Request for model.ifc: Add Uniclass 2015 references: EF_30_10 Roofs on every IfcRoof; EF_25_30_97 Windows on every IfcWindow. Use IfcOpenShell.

First a look at what the model holds.

```python
import ifcopenshell

model = ifcopenshell.open("model.ifc")
print(model.schema)
print("classifications:", [c.Name for c in model.by_type("IfcClassification")])
for ifc_class in ("IfcDoor", "IfcRoof", "IfcStair", "IfcWall", "IfcWindow"):
    print(ifc_class, len(model.by_type(ifc_class)))
```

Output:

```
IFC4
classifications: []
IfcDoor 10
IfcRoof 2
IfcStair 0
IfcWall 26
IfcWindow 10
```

```python
import ifcopenshell
import ifcopenshell.api.classification

model = ifcopenshell.open("model.ifc")

system = ifcopenshell.api.classification.add_classification(model, classification="Uniclass 2015")

codes = {
    "IfcRoof": ("EF_30_10", "Roofs"),
    "IfcWindow": ("EF_25_30_97", "Windows"),
}
for ifc_class, (code, name) in codes.items():
    products = model.by_type(ifc_class)
    ifcopenshell.api.classification.add_reference(
        model, products=products, classification=system, identification=code, name=name
    )
    print(code, len(products))

model.write("model_v2.ifc")
```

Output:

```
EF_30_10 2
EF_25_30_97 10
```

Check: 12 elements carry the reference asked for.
